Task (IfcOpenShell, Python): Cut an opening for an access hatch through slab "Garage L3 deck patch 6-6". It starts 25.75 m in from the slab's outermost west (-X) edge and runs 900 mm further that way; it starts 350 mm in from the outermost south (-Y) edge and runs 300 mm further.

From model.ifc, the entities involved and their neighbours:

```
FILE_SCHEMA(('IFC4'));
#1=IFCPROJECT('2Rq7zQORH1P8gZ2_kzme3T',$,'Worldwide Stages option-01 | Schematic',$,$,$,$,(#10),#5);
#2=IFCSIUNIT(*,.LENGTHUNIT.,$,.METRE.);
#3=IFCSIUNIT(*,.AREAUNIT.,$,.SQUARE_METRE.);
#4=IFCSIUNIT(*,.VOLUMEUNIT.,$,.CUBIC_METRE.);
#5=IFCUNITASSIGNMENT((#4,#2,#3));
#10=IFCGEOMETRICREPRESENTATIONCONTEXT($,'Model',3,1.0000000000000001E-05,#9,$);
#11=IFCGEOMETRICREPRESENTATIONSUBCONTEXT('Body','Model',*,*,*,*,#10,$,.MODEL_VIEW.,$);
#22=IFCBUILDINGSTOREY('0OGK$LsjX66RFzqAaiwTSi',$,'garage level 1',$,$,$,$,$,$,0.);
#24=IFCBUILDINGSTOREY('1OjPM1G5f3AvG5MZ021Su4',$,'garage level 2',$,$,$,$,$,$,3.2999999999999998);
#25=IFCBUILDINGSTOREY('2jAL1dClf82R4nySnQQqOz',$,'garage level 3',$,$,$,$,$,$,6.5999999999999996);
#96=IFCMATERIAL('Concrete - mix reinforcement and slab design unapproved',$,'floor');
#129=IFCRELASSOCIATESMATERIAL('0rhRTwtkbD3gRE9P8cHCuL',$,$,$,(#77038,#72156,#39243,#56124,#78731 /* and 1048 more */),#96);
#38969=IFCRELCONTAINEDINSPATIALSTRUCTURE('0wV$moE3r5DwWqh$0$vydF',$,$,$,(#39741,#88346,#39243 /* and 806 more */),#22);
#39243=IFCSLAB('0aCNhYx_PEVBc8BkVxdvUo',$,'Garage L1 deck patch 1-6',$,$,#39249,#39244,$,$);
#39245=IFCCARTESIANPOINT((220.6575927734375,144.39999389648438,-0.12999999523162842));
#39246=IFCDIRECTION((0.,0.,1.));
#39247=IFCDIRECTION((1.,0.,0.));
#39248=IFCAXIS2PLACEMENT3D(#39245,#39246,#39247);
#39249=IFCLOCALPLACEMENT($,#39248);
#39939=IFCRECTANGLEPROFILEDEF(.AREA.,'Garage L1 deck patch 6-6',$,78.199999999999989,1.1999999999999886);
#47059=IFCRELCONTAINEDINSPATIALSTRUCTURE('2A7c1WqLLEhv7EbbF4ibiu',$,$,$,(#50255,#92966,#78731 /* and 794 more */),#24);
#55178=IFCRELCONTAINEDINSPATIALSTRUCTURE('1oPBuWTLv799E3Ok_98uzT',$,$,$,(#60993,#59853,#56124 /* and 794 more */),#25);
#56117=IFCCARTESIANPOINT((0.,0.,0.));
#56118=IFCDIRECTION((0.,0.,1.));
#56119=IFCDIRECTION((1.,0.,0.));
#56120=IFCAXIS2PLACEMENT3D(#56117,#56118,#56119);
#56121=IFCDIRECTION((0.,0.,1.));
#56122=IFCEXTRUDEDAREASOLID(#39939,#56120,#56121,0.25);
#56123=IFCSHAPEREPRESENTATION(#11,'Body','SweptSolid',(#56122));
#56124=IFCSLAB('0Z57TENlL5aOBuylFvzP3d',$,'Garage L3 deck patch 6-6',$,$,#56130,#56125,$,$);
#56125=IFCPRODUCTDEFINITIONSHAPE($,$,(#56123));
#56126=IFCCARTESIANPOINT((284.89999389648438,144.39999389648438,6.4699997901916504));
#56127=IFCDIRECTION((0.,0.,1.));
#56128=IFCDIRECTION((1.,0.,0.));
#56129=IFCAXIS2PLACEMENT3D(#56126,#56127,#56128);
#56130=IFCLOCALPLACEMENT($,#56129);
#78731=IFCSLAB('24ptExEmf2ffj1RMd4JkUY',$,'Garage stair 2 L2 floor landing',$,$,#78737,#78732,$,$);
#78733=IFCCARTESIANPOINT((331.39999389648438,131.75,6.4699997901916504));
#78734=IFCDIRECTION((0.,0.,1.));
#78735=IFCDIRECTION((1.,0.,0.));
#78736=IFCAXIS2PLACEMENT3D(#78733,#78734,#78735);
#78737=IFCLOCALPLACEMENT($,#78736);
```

```python
import numpy as np
import ifcopenshell
import ifcopenshell.api.feature
import ifcopenshell.api.geometry
import ifcopenshell.api.root
import ifcopenshell.geom
import ifcopenshell.util.placement
import ifcopenshell.util.representation
import ifcopenshell.util.shape
import ifcopenshell.util.unit

model = ifcopenshell.open("model.ifc")
unit_scale = ifcopenshell.util.unit.calculate_unit_scale(model)
settings = ifcopenshell.geom.settings()


def volume(element):
    """Net volume in cubic metres, openings subtracted."""
    shape = ifcopenshell.geom.create_shape(settings, element)
    return ifcopenshell.util.shape.get_volume(shape.geometry)


slab = model.by_guid("0Z57TENlL5aOBuylFvzP3d")
before = volume(slab)

# Extent in the slab's own axes, in metres. The edges named are its -X and -Y sides.
slab_shape = ifcopenshell.geom.create_shape(settings, slab)
vertices = ifcopenshell.util.shape.get_vertices(slab_shape.geometry)
x_min, y_min, bottom = vertices.min(axis=0)
top = vertices[:, 2].max()

opening = ifcopenshell.api.root.create_entity(model, ifc_class="IfcOpeningElement", name="Access hatch opening", predefined_type="OPENING")
context = ifcopenshell.util.representation.get_context(model, "Model", "Body", "MODEL_VIEW")
width, depth = 0.9, 0.3
outline = [(0.0, 0.0), (width, 0.0), (width, depth), (0.0, depth), (0.0, 0.0)]
# Overshoot both faces by 50 mm so the cut is clean.
shape = ifcopenshell.api.geometry.add_slab_representation(
    model, context=context, depth=top - bottom + 0.1, polyline=outline
)
ifcopenshell.api.geometry.assign_representation(model, product=opening, representation=shape)

matrix = ifcopenshell.util.placement.get_local_placement(slab.ObjectPlacement)
matrix[:, 3] = matrix @ np.append(np.array([x_min + 25.75, y_min + 0.35, bottom - 0.05]) / unit_scale, 1.0)
ifcopenshell.api.geometry.edit_object_placement(model, product=opening, matrix=matrix, is_si=False)
ifcopenshell.api.feature.add_feature(model, feature=opening, element=slab)

after = volume(slab)

print(f"slab volume {before:.3f} -> {after:.3f} m3")

model.write("model_rev.ifc")
```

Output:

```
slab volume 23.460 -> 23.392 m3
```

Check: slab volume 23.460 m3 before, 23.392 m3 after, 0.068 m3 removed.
